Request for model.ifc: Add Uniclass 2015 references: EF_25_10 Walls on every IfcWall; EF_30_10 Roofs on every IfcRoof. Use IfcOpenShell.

First a look at what the model holds.

```python
import ifcopenshell

model = ifcopenshell.open("model.ifc")
print(model.schema)
print("classifications:", [c.Name for c in model.by_type("IfcClassification")])
for ifc_class in ("IfcDoor", "IfcRoof", "IfcStair", "IfcWall", "IfcWindow"):
    print(ifc_class, len(model.by_type(ifc_class)))
```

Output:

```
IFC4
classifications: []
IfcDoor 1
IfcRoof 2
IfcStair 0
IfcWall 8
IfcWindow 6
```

```python
import ifcopenshell
import ifcopenshell.api.classification

model = ifcopenshell.open("model.ifc")

system = ifcopenshell.api.classification.add_classification(model, classification="Uniclass 2015")

codes = {
    "IfcWall": ("EF_25_10", "Walls"),
    "IfcRoof": ("EF_30_10", "Roofs"),
}
for ifc_class, (code, name) in codes.items():
    products = model.by_type(ifc_class)
    ifcopenshell.api.classification.add_reference(
        model, products=products, classification=system, identification=code, name=name
    )
    print(code, len(products))

model.write("model_rev.ifc")
```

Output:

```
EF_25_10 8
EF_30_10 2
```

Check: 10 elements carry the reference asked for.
